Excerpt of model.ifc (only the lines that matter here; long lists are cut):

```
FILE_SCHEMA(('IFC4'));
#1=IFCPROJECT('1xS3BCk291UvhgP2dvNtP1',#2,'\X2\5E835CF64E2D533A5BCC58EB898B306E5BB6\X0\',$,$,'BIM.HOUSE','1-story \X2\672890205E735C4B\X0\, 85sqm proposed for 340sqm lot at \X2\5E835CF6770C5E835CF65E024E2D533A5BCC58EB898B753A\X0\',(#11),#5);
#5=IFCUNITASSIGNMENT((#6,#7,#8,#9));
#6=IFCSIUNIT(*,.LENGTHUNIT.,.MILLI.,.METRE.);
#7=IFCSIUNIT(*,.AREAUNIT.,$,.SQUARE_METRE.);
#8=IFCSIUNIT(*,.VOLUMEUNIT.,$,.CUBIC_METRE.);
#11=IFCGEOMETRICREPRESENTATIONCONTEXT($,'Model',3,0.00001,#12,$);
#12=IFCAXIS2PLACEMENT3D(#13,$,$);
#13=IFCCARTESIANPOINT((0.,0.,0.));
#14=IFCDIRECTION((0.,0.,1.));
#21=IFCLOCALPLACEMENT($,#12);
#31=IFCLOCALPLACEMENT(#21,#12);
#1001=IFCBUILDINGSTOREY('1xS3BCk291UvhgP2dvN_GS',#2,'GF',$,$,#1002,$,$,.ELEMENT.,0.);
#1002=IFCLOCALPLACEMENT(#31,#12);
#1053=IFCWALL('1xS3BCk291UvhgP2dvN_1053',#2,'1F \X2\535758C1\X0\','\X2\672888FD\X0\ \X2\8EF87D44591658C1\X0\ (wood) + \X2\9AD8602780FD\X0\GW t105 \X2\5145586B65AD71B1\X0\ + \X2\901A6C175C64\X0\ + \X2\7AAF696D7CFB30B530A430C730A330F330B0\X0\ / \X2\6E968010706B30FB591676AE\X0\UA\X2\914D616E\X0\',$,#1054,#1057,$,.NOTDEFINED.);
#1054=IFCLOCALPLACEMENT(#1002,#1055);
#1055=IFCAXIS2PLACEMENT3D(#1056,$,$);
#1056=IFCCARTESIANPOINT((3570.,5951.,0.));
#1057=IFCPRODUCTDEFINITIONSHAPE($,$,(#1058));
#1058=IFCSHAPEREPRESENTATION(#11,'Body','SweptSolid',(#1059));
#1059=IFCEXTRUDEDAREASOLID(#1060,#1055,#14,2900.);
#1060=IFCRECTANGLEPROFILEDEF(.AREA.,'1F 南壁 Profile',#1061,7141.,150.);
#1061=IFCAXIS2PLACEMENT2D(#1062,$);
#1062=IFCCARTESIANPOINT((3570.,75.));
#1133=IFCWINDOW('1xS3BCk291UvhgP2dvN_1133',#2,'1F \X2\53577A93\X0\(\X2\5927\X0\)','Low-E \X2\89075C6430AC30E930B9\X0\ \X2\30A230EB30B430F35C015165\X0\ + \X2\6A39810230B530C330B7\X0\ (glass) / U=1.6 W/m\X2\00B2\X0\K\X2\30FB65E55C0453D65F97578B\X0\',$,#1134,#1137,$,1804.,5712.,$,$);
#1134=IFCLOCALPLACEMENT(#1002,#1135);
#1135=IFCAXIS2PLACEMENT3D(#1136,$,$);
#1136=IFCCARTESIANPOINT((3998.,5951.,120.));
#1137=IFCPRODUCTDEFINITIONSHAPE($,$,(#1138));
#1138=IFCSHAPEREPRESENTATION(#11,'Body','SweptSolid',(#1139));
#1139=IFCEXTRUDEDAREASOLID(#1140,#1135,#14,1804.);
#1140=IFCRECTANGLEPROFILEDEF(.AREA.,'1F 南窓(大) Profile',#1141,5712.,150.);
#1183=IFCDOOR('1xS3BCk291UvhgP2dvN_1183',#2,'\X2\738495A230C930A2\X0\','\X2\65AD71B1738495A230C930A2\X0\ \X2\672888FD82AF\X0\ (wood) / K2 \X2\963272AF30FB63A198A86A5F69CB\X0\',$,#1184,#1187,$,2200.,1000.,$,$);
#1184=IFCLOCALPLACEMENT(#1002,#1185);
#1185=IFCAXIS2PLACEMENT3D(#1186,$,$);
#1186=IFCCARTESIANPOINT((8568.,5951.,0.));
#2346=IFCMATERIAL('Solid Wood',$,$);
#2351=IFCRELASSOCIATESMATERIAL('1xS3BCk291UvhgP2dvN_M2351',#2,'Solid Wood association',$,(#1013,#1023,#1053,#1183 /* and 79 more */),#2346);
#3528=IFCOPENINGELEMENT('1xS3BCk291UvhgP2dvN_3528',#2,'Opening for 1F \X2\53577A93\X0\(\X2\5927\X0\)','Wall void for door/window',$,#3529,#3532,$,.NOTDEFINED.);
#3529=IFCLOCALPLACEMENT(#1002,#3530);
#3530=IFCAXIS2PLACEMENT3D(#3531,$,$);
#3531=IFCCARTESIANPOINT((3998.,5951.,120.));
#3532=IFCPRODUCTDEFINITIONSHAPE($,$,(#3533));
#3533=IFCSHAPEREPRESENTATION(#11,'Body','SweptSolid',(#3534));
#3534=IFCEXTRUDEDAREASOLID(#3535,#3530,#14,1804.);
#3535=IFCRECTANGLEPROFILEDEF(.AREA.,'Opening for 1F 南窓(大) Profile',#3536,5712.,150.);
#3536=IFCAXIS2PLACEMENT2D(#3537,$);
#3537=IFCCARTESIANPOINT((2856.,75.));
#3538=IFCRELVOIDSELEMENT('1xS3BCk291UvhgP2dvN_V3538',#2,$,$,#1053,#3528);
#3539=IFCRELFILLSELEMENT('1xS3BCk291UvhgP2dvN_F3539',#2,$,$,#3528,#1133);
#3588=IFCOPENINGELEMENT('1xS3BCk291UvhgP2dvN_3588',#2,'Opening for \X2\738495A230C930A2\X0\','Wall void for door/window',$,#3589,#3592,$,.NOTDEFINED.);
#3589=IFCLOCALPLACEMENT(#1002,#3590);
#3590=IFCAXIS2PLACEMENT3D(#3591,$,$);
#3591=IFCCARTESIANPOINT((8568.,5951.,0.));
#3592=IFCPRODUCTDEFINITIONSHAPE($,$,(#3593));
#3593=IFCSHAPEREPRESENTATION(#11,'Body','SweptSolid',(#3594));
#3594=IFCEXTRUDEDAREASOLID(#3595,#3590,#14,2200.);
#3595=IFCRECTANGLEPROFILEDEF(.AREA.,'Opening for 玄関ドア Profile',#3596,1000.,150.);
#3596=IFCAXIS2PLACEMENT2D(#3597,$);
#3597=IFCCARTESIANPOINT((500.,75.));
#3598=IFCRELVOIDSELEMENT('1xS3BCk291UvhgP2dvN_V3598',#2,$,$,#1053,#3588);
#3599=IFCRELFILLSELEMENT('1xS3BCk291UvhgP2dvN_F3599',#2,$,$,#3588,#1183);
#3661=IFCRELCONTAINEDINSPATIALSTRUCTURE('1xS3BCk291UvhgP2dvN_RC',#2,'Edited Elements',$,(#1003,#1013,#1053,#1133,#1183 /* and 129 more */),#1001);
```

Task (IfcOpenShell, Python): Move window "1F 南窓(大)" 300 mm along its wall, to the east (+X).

```python
import ifcopenshell
import ifcopenshell.api.geometry
import ifcopenshell.util.placement

model = ifcopenshell.open("model.ifc")

window = model.by_guid("1xS3BCk291UvhgP2dvN_1133")
opening = window.FillsVoids[0].RelatingOpeningElement
wall = opening.VoidsElements[0].RelatingBuildingElement

wall_matrix = ifcopenshell.util.placement.get_local_placement(wall.ObjectPlacement)
shift = wall_matrix[:3, 0] * 300.0
before = ifcopenshell.util.placement.get_local_placement(window.ObjectPlacement)[:3, 3].copy()

# The window is not placed relative to its opening, so move both.
for product in (opening, window):
    matrix = ifcopenshell.util.placement.get_local_placement(product.ObjectPlacement)
    matrix[:3, 3] += shift
    ifcopenshell.api.geometry.edit_object_placement(model, product=product, matrix=matrix, is_si=False)

after = ifcopenshell.util.placement.get_local_placement(window.ObjectPlacement)[:3, 3]
print("window moved by", (after - before).round(3) + 0.0)

model.write("model_edited.ifc")
```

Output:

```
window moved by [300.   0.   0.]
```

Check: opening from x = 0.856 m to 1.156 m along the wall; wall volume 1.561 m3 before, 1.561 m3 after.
